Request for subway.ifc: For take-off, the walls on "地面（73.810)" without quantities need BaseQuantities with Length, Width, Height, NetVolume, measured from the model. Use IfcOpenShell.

First a look at what the model holds.

```python
import ifcopenshell
import ifcopenshell.util.element
import ifcopenshell.util.unit

model = ifcopenshell.open("subway.ifc")
print(model.schema)
for unit_type in ("LENGTHUNIT", "AREAUNIT", "VOLUMEUNIT"):
    print(unit_type, ifcopenshell.util.unit.calculate_unit_scale(model, unit_type))
storey = next(s for s in model.by_type("IfcBuildingStorey") if s.Name == "地面（73.810)")
walls = [e for e in ifcopenshell.util.element.get_decomposition(storey) if e.is_a("IfcWall")]
for e in sorted(walls, key=lambda e: e.id()):
    print(e.id(), e.is_a(), e.Name, list(ifcopenshell.util.element.get_psets(e, qtos_only=True)), sep=" | ")
```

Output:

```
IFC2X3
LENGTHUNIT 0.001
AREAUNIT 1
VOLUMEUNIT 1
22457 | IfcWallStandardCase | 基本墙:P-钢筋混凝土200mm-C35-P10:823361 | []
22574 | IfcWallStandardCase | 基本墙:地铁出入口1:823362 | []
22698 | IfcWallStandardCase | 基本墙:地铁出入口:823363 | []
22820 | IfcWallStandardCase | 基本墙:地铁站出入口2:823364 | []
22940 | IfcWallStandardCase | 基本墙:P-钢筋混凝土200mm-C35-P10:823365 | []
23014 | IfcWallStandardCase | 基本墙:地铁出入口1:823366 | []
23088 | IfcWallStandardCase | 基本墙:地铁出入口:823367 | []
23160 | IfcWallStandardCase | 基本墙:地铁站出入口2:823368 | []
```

```python
import ifcopenshell
import ifcopenshell.api.pset
import ifcopenshell.geom
import ifcopenshell.util.element
import ifcopenshell.util.shape
import ifcopenshell.util.unit

model = ifcopenshell.open("subway.ifc")
unit_scale = ifcopenshell.util.unit.calculate_unit_scale(model)
volume_scale = ifcopenshell.util.unit.calculate_unit_scale(model, "VOLUMEUNIT")
settings = ifcopenshell.geom.settings()

storey = next(s for s in model.by_type("IfcBuildingStorey") if s.Name == "地面（73.810)")
walls = [e for e in ifcopenshell.util.element.get_decomposition(storey) if e.is_a("IfcWall")]

for e in sorted(walls, key=lambda e: e.id()):
    if ifcopenshell.util.element.get_psets(e, qtos_only=True, should_inherit=False):
        continue
    # Geometry comes back in metres, in the element's own axes.
    shape = ifcopenshell.geom.create_shape(settings, e)
    values = {
        "Length": ifcopenshell.util.shape.get_x(shape.geometry) / unit_scale,
        "Width": ifcopenshell.util.shape.get_y(shape.geometry) / unit_scale,
        "Height": ifcopenshell.util.shape.get_z(shape.geometry) / unit_scale,
        "NetVolume": ifcopenshell.util.shape.get_volume(shape.geometry) / volume_scale,
    }
    qto = ifcopenshell.api.pset.add_qto(model, product=e, name="BaseQuantities")
    ifcopenshell.api.pset.edit_qto(model, qto=qto, properties=values)
    print(e.id(), {k: round(v, 3) for k, v in values.items()})

model.write("subway_edited.ifc")
```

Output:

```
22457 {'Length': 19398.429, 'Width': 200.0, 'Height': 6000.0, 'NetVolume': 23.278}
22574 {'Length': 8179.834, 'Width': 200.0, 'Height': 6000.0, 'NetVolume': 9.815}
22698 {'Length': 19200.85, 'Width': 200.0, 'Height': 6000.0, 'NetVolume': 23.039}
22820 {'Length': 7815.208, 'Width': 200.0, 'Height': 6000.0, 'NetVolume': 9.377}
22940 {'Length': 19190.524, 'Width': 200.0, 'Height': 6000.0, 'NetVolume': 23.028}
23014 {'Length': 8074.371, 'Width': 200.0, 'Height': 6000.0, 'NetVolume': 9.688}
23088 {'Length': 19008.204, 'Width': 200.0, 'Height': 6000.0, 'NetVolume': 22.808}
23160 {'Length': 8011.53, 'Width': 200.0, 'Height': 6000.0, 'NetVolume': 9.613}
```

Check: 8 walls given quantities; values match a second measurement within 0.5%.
